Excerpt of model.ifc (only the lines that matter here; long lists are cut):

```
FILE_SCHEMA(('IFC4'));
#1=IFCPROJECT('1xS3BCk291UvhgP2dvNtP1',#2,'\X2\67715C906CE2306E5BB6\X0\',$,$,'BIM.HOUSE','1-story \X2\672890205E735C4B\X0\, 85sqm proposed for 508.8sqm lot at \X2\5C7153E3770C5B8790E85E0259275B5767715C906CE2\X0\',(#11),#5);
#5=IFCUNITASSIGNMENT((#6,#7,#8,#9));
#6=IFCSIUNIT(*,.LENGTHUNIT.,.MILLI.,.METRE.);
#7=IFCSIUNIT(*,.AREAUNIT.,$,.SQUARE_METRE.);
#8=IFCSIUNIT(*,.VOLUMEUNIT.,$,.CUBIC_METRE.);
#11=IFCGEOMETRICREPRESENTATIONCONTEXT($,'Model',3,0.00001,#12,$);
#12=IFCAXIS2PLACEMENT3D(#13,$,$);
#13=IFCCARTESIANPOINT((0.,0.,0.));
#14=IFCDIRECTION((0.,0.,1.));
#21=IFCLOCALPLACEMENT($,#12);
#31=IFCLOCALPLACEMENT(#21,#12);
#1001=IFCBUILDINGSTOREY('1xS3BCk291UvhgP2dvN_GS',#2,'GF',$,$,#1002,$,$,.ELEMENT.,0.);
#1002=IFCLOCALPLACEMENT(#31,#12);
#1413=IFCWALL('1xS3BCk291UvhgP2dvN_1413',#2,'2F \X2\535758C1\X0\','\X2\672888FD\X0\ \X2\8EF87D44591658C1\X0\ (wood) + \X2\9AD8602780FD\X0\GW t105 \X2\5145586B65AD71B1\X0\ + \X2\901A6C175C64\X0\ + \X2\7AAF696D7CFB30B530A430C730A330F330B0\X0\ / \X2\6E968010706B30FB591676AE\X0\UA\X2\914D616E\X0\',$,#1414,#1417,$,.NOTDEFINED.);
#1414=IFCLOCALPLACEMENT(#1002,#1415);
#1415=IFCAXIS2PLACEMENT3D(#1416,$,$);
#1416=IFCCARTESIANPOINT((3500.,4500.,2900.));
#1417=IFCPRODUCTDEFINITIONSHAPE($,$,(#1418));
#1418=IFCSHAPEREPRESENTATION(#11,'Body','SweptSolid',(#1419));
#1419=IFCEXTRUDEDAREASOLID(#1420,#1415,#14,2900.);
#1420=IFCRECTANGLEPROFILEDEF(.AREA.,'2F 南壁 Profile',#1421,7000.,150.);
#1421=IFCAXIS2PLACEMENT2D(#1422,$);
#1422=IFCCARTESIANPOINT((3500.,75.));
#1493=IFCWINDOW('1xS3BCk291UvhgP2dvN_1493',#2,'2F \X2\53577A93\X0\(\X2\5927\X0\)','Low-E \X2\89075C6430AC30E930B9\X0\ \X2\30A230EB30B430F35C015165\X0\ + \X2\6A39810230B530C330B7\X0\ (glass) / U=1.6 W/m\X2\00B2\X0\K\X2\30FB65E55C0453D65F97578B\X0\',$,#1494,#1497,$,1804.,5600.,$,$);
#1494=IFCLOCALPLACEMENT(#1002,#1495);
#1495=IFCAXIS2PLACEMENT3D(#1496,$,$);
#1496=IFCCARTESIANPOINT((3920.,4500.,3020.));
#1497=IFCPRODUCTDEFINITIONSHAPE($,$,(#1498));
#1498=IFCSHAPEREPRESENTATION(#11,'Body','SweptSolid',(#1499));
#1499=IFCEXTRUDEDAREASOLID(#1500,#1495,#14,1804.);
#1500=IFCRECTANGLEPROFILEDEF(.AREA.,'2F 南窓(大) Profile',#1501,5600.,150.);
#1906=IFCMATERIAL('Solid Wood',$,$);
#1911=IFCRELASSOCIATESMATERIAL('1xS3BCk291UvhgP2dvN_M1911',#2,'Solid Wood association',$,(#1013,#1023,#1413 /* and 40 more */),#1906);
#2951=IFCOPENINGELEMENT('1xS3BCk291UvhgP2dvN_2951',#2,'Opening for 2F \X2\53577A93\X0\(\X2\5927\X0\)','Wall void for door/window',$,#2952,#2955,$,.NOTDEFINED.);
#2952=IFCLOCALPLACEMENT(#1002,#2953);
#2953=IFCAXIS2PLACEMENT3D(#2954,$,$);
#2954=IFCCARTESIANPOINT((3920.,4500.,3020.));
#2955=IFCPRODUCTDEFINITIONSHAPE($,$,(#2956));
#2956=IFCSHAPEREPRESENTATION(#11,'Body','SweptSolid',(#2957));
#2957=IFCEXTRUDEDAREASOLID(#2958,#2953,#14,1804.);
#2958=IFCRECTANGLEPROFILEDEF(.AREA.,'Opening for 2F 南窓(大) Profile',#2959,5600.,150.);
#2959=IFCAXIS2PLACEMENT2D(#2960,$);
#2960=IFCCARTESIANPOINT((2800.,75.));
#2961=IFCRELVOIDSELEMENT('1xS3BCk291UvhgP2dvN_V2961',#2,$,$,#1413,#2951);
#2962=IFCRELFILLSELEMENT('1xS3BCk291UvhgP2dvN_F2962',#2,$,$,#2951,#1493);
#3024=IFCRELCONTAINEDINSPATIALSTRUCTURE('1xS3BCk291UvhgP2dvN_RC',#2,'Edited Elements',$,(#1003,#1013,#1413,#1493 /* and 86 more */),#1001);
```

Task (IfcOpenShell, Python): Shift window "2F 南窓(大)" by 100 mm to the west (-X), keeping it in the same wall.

```python
import ifcopenshell
import ifcopenshell.api.geometry
import ifcopenshell.util.placement

model = ifcopenshell.open("model.ifc")

window = model.by_guid("1xS3BCk291UvhgP2dvN_1493")
opening = window.FillsVoids[0].RelatingOpeningElement
wall = opening.VoidsElements[0].RelatingBuildingElement

wall_matrix = ifcopenshell.util.placement.get_local_placement(wall.ObjectPlacement)
shift = wall_matrix[:3, 0] * -100.0
before = ifcopenshell.util.placement.get_local_placement(window.ObjectPlacement)[:3, 3].copy()

# The window is not placed relative to its opening, so move both.
for product in (opening, window):
    matrix = ifcopenshell.util.placement.get_local_placement(product.ObjectPlacement)
    matrix[:3, 3] += shift
    ifcopenshell.api.geometry.edit_object_placement(model, product=product, matrix=matrix, is_si=False)

after = ifcopenshell.util.placement.get_local_placement(window.ObjectPlacement)[:3, 3]
print("window moved by", (after - before).round(3) + 0.0)

model.write("model-out.ifc")
```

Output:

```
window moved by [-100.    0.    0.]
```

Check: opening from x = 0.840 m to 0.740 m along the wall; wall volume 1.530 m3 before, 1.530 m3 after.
